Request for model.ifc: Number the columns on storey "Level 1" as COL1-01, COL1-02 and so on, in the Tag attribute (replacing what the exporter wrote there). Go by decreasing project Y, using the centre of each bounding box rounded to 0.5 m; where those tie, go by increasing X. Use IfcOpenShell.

First a look at what the model holds.

```python
import ifcopenshell
import ifcopenshell.util.element
import ifcopenshell.util.placement

model = ifcopenshell.open("model.ifc")
print(model.schema)
storey = next(s for s in model.by_type("IfcBuildingStorey") if s.Name == "Level 1")
columns = [e for e in ifcopenshell.util.element.get_decomposition(storey) if e.is_a("IfcColumn")]
for e in sorted(columns, key=lambda e: e.id()):
    origin = ifcopenshell.util.placement.get_local_placement(e.ObjectPlacement)[:3, 3]
    print(e.id(), e.Tag, e.Name, origin.round(2) + 0.0, sep=" | ")
```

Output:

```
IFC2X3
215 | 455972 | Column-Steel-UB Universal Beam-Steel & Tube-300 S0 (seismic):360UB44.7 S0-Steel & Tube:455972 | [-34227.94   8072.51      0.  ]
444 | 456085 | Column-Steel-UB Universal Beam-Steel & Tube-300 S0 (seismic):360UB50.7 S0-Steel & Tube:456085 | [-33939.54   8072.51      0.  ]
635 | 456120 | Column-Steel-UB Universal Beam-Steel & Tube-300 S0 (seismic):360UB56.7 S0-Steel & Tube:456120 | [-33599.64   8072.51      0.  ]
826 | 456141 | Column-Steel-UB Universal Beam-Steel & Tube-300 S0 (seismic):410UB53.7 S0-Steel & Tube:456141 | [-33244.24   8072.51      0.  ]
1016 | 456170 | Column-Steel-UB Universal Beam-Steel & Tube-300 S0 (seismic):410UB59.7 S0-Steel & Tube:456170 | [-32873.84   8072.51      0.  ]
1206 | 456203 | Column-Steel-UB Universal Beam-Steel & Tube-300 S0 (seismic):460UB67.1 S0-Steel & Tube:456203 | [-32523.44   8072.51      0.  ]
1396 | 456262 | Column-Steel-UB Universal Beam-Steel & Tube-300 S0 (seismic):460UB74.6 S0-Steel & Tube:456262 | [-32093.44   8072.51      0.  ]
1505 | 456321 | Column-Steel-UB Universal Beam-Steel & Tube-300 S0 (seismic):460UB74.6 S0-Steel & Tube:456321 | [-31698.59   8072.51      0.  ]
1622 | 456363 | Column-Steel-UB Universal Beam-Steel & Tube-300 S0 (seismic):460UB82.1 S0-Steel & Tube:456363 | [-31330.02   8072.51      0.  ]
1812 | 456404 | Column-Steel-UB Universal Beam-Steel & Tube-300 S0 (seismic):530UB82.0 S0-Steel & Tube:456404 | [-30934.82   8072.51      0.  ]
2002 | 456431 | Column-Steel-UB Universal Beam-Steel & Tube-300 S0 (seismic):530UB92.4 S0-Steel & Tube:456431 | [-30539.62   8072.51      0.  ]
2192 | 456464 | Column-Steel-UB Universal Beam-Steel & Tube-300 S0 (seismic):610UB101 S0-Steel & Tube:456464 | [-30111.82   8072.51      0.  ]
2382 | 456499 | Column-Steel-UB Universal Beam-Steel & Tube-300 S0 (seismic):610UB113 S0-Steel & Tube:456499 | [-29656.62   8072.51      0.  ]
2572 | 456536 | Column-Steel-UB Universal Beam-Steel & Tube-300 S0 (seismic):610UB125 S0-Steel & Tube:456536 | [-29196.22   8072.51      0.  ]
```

```python
import ifcopenshell
import ifcopenshell.geom
import ifcopenshell.util.element
import ifcopenshell.util.shape

model = ifcopenshell.open("model.ifc")
settings = ifcopenshell.geom.settings()
settings.set("use-world-coords", True)


def centre(element):
    shape = ifcopenshell.geom.create_shape(settings, element)
    return ifcopenshell.util.shape.get_bbox_centroid(shape.geometry)


storey = next(s for s in model.by_type("IfcBuildingStorey") if s.Name == "Level 1")
columns = [e for e in ifcopenshell.util.element.get_decomposition(storey) if e.is_a("IfcColumn")]

# Insertion points can sit at a corner or the storey origin, so sort by the geometry (in metres).
centres = {e: centre(e) for e in columns}
columns.sort(key=lambda e: (-round(centres[e][1] / 0.5), centres[e][0]))

for i, e in enumerate(columns, start=1):
    number = f"COL1-{i:02d}"
    e.Tag = number
    print(e.id(), number)

model.write("model_v2.ifc")
```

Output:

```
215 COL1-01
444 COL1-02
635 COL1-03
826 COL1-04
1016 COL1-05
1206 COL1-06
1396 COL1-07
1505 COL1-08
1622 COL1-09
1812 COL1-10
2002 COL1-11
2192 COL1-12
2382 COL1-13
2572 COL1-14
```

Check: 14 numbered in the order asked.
